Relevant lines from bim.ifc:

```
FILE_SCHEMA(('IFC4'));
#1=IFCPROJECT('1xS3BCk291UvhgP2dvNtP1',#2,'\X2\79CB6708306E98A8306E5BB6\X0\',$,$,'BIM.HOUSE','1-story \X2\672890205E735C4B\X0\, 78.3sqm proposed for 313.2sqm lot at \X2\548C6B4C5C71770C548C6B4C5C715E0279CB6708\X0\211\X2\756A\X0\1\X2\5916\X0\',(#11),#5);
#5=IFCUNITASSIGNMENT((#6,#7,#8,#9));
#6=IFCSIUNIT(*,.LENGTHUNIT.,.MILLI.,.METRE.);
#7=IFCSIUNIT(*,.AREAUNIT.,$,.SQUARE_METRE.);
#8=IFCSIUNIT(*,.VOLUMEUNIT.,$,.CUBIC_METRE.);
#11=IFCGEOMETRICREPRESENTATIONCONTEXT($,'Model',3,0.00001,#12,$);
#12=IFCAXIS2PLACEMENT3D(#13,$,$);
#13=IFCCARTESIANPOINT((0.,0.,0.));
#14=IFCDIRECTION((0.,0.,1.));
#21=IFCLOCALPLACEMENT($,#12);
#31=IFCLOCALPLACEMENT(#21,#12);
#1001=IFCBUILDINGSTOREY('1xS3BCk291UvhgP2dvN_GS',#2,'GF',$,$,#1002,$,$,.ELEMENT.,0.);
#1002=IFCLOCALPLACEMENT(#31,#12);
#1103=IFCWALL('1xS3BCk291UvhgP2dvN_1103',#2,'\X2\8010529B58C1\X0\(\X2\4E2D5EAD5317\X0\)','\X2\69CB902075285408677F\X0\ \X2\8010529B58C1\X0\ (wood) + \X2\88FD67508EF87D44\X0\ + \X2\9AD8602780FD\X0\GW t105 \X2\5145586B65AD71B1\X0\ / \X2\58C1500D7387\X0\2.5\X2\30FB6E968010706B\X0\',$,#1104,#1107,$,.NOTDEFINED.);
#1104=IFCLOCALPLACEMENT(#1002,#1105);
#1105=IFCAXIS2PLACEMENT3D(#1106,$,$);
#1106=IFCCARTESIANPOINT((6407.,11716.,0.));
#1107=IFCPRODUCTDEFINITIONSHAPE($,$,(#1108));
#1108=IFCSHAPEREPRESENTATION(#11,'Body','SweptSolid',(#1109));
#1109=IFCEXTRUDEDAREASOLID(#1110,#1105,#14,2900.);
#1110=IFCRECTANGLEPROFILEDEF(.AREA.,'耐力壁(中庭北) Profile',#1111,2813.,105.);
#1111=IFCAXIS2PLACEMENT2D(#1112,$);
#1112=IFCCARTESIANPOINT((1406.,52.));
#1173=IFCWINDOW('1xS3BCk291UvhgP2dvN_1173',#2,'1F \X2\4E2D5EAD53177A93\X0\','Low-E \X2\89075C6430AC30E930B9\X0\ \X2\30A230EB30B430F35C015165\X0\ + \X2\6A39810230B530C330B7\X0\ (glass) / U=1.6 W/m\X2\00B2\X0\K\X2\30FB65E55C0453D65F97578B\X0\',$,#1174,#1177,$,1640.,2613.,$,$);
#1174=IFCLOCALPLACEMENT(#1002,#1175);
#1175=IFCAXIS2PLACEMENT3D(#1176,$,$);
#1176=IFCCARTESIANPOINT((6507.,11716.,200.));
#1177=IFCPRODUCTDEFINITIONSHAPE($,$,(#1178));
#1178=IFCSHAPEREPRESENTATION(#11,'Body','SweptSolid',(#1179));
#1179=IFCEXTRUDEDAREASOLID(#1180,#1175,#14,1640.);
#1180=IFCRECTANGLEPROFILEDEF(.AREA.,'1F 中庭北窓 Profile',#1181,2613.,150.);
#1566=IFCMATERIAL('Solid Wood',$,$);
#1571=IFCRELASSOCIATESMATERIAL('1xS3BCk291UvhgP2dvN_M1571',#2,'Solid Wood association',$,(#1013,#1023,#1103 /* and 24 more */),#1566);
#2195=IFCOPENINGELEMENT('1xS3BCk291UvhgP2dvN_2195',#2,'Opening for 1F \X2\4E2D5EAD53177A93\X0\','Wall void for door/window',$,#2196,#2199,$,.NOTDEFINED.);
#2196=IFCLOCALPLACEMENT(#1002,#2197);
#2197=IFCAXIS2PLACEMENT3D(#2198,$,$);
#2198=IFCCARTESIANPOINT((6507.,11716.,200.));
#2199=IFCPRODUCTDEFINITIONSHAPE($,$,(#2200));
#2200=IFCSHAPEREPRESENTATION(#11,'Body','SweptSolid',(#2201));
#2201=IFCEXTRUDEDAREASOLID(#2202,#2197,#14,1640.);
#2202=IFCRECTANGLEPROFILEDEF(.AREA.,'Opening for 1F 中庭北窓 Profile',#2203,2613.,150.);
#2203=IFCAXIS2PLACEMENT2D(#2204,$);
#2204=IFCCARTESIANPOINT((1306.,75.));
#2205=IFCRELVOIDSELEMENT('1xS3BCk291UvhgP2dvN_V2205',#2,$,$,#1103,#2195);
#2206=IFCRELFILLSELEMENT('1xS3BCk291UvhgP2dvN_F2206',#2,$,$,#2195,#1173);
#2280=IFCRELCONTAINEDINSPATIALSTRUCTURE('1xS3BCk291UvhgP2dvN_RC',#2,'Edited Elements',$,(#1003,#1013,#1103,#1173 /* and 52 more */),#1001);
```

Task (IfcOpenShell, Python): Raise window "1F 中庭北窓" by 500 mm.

```python
import numpy as np
import ifcopenshell
import ifcopenshell.api.geometry
import ifcopenshell.util.placement
import ifcopenshell.util.unit

model = ifcopenshell.open("bim.ifc")
unit_scale = ifcopenshell.util.unit.calculate_unit_scale(model)

window = model.by_id(1173)
opening = window.FillsVoids[0].RelatingOpeningElement
dz = 500.0

shift = np.array([0.0, 0.0, dz])
# The window is not placed relative to its opening, so move both.
for product in (opening, window):
    matrix = ifcopenshell.util.placement.get_local_placement(product.ObjectPlacement)
    matrix[:3, 3] += shift
    ifcopenshell.api.geometry.edit_object_placement(model, product=product, matrix=matrix, is_si=False)

print(f"moved by {dz * unit_scale:+.3f} m")

model.write("bim_updated.ifc")
```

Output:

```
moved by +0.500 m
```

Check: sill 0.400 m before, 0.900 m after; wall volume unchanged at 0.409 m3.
